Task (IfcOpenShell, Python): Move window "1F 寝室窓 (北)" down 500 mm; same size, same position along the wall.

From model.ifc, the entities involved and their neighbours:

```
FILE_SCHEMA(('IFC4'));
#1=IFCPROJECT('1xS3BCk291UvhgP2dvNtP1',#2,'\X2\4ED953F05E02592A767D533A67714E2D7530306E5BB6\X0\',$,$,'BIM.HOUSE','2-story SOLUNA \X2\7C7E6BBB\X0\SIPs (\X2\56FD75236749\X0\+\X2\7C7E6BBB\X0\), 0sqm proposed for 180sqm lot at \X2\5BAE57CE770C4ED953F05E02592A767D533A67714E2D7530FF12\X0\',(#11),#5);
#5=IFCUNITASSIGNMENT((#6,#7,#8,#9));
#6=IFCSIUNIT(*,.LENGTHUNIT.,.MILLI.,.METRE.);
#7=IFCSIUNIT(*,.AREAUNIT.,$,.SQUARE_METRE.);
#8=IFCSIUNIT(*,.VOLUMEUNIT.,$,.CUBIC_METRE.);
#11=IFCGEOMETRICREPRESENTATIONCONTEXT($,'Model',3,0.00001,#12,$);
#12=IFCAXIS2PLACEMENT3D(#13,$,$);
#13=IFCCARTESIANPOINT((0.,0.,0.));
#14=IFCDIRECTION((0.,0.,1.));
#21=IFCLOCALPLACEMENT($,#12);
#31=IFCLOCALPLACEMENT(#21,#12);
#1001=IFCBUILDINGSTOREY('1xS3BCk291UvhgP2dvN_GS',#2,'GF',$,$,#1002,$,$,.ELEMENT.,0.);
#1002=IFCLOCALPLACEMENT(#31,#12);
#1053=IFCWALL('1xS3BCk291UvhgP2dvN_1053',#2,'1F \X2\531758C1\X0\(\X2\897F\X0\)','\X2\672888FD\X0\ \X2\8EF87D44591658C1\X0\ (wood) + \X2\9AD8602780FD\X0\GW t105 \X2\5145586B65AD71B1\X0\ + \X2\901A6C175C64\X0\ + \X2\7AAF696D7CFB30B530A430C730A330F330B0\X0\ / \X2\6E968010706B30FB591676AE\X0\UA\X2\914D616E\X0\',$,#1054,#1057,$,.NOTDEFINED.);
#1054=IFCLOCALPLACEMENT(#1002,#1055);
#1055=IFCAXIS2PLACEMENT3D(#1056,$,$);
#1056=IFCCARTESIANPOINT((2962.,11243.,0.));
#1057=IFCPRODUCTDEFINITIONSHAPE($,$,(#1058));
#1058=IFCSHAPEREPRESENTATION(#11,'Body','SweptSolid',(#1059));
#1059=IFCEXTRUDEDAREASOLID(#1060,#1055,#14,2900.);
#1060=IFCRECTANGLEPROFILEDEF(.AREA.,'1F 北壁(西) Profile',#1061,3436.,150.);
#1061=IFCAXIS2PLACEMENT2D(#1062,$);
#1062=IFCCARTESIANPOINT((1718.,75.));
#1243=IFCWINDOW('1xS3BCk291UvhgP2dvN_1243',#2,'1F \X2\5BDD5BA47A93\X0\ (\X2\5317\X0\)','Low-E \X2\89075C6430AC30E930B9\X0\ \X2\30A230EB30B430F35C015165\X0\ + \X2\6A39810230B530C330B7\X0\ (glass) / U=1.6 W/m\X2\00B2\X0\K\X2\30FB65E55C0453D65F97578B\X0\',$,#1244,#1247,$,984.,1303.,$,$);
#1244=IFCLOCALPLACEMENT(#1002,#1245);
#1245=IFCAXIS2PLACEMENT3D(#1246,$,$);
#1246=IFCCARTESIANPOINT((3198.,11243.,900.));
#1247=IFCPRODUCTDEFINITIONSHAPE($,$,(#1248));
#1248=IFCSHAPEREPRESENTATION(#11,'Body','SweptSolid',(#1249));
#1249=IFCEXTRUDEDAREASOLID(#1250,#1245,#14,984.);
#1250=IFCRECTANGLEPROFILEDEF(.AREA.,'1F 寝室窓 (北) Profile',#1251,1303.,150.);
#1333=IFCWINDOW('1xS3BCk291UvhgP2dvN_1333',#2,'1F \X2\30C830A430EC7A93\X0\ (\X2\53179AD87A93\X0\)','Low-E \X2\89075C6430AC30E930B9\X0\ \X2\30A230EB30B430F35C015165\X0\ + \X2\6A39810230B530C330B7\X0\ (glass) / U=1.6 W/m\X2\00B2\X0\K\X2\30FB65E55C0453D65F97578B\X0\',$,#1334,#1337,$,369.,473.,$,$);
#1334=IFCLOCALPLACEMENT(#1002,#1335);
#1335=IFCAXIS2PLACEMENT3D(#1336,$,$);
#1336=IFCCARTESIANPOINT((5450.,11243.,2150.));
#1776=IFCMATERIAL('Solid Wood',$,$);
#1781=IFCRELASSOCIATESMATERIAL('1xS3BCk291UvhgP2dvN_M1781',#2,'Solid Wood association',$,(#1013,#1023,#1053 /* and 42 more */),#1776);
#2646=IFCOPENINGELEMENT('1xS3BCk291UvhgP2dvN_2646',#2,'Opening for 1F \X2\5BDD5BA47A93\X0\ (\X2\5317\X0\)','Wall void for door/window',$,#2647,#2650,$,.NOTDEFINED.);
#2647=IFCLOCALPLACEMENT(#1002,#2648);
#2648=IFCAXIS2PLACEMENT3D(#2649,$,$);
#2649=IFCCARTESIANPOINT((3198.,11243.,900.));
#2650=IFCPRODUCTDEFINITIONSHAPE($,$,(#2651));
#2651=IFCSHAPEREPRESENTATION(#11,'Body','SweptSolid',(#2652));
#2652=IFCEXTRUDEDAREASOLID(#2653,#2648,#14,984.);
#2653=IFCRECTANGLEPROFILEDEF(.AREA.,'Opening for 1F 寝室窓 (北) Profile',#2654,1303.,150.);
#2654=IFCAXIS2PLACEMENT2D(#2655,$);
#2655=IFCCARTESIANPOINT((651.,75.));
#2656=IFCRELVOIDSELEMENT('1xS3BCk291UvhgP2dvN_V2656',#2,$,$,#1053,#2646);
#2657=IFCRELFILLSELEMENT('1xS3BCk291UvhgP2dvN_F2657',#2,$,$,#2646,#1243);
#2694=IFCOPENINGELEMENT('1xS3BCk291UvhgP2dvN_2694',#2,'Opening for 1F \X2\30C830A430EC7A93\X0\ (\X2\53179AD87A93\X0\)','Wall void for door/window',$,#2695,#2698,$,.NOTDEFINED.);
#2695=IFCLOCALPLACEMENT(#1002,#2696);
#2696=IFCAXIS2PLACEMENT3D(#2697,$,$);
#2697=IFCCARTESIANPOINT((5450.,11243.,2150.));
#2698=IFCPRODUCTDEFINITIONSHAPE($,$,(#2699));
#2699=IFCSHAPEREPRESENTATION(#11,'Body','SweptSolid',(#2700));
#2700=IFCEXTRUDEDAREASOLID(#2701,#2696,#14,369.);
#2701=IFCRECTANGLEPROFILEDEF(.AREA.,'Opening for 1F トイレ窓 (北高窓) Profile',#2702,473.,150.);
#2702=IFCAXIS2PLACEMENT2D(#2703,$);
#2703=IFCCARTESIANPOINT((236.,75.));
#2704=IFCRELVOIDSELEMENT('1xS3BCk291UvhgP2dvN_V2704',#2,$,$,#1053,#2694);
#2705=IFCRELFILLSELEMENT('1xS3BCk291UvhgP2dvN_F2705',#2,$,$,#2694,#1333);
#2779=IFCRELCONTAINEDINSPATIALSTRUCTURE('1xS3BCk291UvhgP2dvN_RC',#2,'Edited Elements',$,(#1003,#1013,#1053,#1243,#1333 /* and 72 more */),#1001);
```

```python
import numpy as np
import ifcopenshell
import ifcopenshell.api.geometry
import ifcopenshell.util.placement
import ifcopenshell.util.unit

model = ifcopenshell.open("model.ifc")
unit_scale = ifcopenshell.util.unit.calculate_unit_scale(model)

window = model.by_guid("1xS3BCk291UvhgP2dvN_1243")
opening = window.FillsVoids[0].RelatingOpeningElement
dz = -500.0

shift = np.array([0.0, 0.0, dz])
# The window is not placed relative to its opening, so move both.
for product in (opening, window):
    matrix = ifcopenshell.util.placement.get_local_placement(product.ObjectPlacement)
    matrix[:3, 3] += shift
    ifcopenshell.api.geometry.edit_object_placement(model, product=product, matrix=matrix, is_si=False)

print(f"moved by {dz * unit_scale:+.3f} m")

model.write("model_edited.ifc")
```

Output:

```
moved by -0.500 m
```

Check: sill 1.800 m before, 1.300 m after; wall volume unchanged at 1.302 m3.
